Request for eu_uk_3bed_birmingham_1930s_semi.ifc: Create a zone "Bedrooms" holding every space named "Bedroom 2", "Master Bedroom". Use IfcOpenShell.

First a look at what the model holds.

```python
import ifcopenshell

model = ifcopenshell.open("eu_uk_3bed_birmingham_1930s_semi.ifc")
print(model.schema)
seen = {}
for space in model.by_type("IfcSpace"):
    seen[space.LongName] = seen.get(space.LongName, 0) + 1
for name, count in sorted(seen.items(), key=str):
    print(count, "x", name)
print("zones:", [z.Name for z in model.by_type("IfcZone")][:20])
```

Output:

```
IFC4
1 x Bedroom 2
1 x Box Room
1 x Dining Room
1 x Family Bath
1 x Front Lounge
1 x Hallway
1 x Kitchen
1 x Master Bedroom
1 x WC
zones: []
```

```python
import ifcopenshell
import ifcopenshell.api.group
import ifcopenshell.api.root

model = ifcopenshell.open("eu_uk_3bed_birmingham_1930s_semi.ifc")

names = {"Bedroom 2", "Master Bedroom"}
spaces = [s for s in model.by_type("IfcSpace") if s.LongName in names]

zone = ifcopenshell.api.root.create_entity(model, ifc_class="IfcZone", name="Bedrooms")
ifcopenshell.api.group.assign_group(model, products=spaces, group=zone)
print(len(spaces), "spaces in", zone.Name)

model.write("eu_uk_3bed_birmingham_1930s_semi-out.ifc")
```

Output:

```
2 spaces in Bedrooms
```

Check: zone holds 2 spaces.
